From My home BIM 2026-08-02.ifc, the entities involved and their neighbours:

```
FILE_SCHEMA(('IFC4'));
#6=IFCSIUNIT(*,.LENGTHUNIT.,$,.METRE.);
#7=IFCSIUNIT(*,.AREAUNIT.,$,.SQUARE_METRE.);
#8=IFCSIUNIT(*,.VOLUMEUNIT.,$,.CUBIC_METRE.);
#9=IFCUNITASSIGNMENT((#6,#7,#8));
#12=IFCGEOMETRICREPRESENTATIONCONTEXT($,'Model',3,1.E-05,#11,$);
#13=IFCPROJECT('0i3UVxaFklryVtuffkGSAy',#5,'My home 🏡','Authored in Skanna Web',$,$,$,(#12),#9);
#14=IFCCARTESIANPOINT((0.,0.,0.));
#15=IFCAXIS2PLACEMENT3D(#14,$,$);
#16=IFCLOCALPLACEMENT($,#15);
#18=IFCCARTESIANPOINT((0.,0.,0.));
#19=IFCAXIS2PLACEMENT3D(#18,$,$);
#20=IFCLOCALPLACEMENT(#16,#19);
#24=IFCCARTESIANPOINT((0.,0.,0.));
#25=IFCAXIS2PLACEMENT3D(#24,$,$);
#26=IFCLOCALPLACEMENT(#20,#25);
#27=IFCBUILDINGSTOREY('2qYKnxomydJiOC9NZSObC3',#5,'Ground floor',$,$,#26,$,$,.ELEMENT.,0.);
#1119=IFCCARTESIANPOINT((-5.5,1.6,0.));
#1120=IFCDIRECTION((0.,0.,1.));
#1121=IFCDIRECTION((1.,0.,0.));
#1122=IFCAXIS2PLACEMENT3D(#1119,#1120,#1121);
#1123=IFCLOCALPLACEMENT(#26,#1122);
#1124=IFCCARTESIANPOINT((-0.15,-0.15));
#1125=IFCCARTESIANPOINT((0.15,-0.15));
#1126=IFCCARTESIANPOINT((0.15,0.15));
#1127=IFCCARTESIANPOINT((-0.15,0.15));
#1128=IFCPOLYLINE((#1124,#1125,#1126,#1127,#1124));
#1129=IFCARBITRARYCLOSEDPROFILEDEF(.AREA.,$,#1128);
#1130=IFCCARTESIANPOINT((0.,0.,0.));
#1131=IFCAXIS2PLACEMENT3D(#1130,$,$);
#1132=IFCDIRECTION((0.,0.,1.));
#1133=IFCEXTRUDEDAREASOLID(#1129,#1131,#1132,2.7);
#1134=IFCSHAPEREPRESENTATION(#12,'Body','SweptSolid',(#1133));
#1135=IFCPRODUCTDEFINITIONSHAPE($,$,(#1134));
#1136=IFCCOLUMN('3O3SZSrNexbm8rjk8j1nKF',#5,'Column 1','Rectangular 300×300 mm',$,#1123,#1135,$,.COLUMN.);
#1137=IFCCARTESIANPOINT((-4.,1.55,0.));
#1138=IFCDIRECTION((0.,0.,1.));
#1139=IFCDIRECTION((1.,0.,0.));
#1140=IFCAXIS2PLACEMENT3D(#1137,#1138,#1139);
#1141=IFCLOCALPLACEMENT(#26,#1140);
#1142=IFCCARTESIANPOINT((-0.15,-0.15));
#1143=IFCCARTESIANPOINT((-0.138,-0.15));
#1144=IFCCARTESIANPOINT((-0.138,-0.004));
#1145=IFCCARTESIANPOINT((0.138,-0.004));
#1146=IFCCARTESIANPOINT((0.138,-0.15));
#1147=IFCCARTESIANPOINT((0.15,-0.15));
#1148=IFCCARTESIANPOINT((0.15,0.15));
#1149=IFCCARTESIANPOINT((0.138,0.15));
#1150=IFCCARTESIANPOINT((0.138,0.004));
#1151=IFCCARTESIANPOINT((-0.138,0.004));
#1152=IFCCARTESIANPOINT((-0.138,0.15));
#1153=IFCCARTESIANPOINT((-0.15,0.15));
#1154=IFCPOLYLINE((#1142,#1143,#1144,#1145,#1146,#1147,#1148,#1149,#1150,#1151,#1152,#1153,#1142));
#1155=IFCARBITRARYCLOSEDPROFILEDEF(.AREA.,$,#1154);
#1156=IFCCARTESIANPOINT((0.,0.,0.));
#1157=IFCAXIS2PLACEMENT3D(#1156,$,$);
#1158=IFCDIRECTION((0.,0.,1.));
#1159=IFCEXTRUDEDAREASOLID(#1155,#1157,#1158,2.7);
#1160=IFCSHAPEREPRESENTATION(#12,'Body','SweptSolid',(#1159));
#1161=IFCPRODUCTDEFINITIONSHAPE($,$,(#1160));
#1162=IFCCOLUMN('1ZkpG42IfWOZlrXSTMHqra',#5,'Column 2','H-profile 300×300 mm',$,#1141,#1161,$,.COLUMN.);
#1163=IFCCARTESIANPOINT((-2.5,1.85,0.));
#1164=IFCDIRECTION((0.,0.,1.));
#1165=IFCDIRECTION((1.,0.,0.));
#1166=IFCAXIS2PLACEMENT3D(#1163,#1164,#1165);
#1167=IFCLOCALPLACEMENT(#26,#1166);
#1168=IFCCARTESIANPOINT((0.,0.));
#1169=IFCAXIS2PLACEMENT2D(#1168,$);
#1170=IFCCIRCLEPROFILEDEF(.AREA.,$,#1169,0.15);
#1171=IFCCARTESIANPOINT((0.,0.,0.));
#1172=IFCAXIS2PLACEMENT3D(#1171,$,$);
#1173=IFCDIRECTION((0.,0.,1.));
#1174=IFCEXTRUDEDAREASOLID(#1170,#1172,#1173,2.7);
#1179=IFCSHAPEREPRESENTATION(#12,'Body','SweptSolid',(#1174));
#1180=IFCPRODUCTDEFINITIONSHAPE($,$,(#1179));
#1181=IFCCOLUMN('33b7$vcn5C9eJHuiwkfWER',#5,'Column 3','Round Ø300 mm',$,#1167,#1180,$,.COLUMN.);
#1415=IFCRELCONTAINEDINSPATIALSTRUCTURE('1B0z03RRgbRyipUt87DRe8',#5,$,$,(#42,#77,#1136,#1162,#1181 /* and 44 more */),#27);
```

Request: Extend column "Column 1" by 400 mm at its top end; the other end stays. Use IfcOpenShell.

```python
import ifcopenshell
import ifcopenshell.util.unit

model = ifcopenshell.open("My home BIM 2026-08-02.ifc")
unit_scale = ifcopenshell.util.unit.calculate_unit_scale(model)

member = model.by_id(1136)
change = 0.4 / unit_scale

# The extrusion runs towards the end named, so only its depth changes.
body = next(r for r in member.Representation.Representations if r.RepresentationIdentifier == "Body")
solid = body.Items[0]
old_length = solid.Depth
solid.Depth += change

print(f"length {old_length:g} -> {solid.Depth:g}")

model.write("My home BIM 2026-08-02_updated.ifc")
```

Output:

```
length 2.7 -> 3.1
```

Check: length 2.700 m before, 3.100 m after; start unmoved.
